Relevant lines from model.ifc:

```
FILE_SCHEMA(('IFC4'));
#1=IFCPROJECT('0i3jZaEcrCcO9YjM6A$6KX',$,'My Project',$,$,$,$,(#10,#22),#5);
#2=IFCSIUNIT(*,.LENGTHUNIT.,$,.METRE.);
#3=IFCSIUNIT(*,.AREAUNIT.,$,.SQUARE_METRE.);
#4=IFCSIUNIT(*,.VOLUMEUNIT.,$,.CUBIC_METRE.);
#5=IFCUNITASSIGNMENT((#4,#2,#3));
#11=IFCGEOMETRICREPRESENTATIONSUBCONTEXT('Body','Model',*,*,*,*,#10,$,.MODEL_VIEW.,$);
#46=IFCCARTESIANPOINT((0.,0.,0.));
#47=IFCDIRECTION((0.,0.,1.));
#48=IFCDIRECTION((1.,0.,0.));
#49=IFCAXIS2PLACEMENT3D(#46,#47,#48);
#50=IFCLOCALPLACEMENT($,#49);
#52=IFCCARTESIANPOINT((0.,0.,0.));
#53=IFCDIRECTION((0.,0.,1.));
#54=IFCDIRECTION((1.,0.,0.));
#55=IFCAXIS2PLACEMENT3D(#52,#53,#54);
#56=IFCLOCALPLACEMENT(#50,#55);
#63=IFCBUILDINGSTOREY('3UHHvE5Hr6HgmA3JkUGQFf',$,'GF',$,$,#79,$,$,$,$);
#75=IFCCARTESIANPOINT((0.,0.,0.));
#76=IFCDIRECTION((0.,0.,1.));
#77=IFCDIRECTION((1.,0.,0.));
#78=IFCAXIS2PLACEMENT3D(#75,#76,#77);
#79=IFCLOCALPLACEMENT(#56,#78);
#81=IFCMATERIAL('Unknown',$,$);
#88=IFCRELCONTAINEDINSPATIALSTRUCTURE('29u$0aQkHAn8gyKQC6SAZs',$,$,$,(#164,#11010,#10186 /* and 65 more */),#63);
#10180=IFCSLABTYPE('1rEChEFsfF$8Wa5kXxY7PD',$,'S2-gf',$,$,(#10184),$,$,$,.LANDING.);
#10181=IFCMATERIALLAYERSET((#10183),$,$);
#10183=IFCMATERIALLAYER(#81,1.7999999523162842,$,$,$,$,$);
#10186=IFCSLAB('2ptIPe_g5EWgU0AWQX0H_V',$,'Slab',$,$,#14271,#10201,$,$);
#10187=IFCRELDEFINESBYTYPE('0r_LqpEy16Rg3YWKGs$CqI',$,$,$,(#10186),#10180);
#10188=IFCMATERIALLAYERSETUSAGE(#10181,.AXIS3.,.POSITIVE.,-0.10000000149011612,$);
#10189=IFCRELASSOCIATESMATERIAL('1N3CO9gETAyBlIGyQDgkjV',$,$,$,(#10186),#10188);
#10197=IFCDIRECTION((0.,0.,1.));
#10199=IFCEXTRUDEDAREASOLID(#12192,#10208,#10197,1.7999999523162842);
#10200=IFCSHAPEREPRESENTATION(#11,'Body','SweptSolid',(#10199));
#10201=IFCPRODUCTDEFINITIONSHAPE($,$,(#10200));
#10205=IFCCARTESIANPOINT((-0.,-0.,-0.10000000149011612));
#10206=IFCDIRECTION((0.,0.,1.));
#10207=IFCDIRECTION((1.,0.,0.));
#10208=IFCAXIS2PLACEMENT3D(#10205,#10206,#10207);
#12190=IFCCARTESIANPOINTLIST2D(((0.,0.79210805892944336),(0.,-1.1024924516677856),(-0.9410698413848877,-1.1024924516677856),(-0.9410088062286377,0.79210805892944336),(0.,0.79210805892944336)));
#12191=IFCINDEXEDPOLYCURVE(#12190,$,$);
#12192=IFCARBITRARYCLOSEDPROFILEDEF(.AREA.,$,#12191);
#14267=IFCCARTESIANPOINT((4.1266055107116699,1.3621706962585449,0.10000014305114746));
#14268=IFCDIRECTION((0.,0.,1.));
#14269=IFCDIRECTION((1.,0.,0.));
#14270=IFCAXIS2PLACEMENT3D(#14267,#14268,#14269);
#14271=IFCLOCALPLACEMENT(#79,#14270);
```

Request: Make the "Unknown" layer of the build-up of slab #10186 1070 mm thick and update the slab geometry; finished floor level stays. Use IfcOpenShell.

```python
import ifcopenshell
import ifcopenshell.util.element
import ifcopenshell.util.representation
import ifcopenshell.util.unit

model = ifcopenshell.open("model.ifc")
unit_scale = ifcopenshell.util.unit.calculate_unit_scale(model)

layer_set = model.by_id(10181)
layer = next(l for l in layer_set.MaterialLayers if l.Material and l.Material.Name == "Unknown")
change = 1.07 / unit_scale - layer.LayerThickness
layer.LayerThickness += change

# Geometry does not follow the layer set by itself.
slabs = [e for e in ifcopenshell.util.element.get_elements_by_material(model, layer_set) if e.is_a("IfcSlab")]
for slab in sorted(slabs, key=lambda e: e.id()):
    body = ifcopenshell.util.representation.get_representation(slab, "Model", "Body")
    solid = body.Items[0]
    old_depth = solid.Depth
    solid.Depth += change
    # Extruded upwards: lower the start of the extrusion so the top stays.
    x, y, z = solid.Position.Location.Coordinates
    solid.Position.Location = model.createIfcCartesianPoint((x, y, z - change))
    print(slab.id(), f"{old_depth:g} -> {solid.Depth:g}")

# The layers are counted up from the underside, which has moved.
for usage in {ifcopenshell.util.element.get_material(slab) for slab in slabs}:
    usage.OffsetFromReferenceLine -= change

model.write("model_rev.ifc")
```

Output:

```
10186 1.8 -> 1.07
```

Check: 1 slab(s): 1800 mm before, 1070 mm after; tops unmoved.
